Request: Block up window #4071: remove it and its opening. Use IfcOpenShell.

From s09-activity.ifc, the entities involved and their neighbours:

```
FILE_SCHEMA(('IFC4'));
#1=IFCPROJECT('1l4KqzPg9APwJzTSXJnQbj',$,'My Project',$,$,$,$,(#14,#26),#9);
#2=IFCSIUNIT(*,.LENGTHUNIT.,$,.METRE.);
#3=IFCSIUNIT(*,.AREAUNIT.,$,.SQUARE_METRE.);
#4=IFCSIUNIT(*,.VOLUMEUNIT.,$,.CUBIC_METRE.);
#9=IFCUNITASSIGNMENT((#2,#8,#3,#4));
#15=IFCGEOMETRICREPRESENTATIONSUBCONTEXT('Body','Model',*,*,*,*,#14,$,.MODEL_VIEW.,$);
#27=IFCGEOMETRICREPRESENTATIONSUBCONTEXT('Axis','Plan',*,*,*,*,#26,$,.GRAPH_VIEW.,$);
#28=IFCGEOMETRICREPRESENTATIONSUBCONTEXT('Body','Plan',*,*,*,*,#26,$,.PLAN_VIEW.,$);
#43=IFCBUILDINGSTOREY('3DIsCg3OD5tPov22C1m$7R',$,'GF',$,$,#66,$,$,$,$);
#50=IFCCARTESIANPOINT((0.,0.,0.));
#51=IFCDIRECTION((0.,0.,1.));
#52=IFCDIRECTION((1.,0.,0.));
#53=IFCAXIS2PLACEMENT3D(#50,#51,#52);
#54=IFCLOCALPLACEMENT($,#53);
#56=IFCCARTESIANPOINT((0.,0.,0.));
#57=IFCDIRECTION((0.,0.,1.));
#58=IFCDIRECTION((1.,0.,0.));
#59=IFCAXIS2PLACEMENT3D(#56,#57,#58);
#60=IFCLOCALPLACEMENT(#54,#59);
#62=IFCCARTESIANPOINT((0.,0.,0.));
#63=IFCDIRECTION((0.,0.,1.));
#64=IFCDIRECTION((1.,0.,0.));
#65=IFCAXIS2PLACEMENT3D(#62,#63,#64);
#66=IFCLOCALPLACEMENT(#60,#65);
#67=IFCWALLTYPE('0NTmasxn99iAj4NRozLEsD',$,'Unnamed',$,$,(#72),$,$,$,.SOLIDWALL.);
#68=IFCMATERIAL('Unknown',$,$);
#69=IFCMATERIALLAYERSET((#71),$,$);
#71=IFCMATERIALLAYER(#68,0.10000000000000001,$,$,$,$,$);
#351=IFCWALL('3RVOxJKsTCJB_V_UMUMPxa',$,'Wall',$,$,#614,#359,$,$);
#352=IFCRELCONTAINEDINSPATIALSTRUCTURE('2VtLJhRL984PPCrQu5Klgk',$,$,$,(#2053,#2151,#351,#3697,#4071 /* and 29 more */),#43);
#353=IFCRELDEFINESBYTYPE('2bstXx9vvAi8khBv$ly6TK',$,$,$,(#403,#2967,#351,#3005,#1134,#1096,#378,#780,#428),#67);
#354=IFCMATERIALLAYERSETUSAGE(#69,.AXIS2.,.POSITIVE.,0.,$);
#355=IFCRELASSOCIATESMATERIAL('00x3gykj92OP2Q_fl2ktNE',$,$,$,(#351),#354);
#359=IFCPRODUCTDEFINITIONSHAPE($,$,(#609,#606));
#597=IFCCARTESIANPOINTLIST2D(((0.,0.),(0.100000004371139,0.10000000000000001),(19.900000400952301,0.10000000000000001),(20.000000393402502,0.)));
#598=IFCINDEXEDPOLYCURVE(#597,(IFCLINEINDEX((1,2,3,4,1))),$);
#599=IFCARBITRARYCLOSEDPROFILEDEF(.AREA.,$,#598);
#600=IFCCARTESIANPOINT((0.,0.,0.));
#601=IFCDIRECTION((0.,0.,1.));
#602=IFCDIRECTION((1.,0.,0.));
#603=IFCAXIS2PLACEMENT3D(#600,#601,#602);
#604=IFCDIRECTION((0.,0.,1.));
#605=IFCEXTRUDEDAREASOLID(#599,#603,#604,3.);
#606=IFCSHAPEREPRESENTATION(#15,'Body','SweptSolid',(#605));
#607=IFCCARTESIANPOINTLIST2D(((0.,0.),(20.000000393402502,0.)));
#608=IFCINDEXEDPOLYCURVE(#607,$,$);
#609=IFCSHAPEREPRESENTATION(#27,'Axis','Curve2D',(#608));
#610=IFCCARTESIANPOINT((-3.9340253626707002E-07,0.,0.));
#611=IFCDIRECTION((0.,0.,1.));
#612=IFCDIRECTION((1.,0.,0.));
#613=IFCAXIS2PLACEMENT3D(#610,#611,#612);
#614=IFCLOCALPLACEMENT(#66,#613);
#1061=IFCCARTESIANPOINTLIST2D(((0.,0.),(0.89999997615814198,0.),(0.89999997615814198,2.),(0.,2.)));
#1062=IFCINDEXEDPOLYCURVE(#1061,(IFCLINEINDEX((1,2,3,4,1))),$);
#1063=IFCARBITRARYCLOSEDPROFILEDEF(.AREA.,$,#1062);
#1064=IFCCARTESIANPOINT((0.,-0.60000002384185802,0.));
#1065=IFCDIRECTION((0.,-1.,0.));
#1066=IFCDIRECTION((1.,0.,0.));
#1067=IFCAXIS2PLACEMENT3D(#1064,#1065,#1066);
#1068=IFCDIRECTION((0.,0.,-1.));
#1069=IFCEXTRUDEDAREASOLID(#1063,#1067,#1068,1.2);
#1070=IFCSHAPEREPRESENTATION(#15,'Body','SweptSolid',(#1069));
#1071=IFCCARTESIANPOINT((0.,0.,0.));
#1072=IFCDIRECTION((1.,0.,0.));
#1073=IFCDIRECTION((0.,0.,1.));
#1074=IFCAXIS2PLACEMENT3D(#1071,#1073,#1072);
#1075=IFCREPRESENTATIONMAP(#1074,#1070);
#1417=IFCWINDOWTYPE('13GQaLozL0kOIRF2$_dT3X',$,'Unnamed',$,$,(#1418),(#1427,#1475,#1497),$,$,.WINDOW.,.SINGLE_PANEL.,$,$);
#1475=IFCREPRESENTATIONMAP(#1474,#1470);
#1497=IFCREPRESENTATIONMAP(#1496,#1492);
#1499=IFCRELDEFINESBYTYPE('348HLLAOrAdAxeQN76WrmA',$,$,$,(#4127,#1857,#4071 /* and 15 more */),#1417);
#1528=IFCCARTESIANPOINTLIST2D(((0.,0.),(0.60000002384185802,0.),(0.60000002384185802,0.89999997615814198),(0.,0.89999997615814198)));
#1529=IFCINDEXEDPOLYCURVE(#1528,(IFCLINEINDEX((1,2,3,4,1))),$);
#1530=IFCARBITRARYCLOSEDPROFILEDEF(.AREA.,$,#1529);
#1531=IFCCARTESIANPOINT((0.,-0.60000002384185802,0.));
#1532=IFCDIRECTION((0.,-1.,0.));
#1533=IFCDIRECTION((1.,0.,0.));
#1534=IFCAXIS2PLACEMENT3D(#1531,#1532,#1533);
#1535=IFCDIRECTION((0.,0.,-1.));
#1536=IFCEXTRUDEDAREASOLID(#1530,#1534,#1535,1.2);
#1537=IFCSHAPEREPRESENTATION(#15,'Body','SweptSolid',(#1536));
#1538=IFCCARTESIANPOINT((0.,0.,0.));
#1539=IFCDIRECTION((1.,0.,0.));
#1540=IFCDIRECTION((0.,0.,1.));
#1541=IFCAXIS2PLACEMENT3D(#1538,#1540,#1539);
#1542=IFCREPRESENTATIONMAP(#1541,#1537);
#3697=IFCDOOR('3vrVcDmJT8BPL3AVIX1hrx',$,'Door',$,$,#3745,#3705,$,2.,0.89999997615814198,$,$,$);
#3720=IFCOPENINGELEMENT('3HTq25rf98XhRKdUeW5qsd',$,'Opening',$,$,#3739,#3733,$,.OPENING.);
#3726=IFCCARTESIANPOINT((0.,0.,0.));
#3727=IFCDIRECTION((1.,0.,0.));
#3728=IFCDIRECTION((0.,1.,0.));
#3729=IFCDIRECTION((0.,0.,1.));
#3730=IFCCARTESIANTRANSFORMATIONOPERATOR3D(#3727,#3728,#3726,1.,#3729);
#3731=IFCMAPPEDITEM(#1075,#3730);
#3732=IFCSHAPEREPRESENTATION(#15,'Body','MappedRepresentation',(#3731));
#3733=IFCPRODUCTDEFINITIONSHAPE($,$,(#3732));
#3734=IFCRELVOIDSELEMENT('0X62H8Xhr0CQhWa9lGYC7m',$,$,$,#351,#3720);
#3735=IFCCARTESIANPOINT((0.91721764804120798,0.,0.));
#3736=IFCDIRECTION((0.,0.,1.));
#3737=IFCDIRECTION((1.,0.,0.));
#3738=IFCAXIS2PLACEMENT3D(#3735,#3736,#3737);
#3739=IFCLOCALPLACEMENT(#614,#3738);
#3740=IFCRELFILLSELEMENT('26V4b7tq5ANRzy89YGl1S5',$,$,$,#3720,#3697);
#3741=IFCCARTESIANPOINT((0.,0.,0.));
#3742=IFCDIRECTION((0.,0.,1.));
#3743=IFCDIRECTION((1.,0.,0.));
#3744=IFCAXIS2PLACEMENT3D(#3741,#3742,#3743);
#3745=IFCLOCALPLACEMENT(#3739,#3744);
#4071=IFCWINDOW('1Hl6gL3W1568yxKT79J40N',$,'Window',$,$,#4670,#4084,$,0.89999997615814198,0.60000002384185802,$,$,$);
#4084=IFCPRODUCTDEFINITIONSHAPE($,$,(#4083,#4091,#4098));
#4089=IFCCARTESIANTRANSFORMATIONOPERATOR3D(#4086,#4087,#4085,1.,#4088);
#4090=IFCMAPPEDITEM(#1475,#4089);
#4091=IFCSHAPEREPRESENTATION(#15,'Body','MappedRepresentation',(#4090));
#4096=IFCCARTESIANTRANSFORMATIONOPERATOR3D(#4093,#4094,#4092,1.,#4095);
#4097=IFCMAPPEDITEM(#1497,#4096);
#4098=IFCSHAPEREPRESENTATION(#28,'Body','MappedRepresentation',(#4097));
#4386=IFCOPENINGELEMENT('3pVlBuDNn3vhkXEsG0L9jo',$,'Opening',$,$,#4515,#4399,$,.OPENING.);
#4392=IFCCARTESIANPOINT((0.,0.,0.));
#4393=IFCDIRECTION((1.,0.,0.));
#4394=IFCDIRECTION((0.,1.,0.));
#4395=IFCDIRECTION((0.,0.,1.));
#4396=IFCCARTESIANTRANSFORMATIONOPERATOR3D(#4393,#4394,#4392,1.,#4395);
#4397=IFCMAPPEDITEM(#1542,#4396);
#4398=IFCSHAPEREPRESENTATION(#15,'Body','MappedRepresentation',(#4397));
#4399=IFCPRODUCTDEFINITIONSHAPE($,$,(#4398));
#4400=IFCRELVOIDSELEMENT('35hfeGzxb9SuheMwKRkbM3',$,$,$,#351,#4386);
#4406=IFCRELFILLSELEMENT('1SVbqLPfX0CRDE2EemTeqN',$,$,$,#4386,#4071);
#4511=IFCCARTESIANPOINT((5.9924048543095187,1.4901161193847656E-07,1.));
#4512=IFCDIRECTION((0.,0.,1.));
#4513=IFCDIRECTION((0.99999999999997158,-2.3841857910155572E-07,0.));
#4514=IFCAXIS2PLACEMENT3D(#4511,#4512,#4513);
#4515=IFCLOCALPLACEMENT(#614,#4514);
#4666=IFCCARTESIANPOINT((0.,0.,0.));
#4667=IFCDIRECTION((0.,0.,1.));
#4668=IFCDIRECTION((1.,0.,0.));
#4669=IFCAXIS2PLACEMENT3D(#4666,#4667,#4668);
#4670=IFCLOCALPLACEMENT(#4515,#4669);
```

```python
import ifcopenshell
import ifcopenshell.api.feature
import ifcopenshell.api.root
import ifcopenshell.geom
import ifcopenshell.util.shape

model = ifcopenshell.open("s09-activity.ifc")
settings = ifcopenshell.geom.settings()


def volume(element):
    """Net volume in cubic metres, openings subtracted."""
    shape = ifcopenshell.geom.create_shape(settings, element)
    return ifcopenshell.util.shape.get_volume(shape.geometry)


window = model.by_guid("1Hl6gL3W1568yxKT79J40N")
opening = window.FillsVoids[0].RelatingOpeningElement
wall = opening.VoidsElements[0].RelatingBuildingElement
before = volume(wall)

ifcopenshell.api.root.remove_product(model, product=window)
ifcopenshell.api.feature.remove_feature(model, feature=opening)

after = volume(wall)

print(f"wall volume {before:.3f} -> {after:.3f} m3")

model.write("s09-activity_updated.ifc")
```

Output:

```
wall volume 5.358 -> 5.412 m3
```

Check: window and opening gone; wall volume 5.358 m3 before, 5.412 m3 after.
